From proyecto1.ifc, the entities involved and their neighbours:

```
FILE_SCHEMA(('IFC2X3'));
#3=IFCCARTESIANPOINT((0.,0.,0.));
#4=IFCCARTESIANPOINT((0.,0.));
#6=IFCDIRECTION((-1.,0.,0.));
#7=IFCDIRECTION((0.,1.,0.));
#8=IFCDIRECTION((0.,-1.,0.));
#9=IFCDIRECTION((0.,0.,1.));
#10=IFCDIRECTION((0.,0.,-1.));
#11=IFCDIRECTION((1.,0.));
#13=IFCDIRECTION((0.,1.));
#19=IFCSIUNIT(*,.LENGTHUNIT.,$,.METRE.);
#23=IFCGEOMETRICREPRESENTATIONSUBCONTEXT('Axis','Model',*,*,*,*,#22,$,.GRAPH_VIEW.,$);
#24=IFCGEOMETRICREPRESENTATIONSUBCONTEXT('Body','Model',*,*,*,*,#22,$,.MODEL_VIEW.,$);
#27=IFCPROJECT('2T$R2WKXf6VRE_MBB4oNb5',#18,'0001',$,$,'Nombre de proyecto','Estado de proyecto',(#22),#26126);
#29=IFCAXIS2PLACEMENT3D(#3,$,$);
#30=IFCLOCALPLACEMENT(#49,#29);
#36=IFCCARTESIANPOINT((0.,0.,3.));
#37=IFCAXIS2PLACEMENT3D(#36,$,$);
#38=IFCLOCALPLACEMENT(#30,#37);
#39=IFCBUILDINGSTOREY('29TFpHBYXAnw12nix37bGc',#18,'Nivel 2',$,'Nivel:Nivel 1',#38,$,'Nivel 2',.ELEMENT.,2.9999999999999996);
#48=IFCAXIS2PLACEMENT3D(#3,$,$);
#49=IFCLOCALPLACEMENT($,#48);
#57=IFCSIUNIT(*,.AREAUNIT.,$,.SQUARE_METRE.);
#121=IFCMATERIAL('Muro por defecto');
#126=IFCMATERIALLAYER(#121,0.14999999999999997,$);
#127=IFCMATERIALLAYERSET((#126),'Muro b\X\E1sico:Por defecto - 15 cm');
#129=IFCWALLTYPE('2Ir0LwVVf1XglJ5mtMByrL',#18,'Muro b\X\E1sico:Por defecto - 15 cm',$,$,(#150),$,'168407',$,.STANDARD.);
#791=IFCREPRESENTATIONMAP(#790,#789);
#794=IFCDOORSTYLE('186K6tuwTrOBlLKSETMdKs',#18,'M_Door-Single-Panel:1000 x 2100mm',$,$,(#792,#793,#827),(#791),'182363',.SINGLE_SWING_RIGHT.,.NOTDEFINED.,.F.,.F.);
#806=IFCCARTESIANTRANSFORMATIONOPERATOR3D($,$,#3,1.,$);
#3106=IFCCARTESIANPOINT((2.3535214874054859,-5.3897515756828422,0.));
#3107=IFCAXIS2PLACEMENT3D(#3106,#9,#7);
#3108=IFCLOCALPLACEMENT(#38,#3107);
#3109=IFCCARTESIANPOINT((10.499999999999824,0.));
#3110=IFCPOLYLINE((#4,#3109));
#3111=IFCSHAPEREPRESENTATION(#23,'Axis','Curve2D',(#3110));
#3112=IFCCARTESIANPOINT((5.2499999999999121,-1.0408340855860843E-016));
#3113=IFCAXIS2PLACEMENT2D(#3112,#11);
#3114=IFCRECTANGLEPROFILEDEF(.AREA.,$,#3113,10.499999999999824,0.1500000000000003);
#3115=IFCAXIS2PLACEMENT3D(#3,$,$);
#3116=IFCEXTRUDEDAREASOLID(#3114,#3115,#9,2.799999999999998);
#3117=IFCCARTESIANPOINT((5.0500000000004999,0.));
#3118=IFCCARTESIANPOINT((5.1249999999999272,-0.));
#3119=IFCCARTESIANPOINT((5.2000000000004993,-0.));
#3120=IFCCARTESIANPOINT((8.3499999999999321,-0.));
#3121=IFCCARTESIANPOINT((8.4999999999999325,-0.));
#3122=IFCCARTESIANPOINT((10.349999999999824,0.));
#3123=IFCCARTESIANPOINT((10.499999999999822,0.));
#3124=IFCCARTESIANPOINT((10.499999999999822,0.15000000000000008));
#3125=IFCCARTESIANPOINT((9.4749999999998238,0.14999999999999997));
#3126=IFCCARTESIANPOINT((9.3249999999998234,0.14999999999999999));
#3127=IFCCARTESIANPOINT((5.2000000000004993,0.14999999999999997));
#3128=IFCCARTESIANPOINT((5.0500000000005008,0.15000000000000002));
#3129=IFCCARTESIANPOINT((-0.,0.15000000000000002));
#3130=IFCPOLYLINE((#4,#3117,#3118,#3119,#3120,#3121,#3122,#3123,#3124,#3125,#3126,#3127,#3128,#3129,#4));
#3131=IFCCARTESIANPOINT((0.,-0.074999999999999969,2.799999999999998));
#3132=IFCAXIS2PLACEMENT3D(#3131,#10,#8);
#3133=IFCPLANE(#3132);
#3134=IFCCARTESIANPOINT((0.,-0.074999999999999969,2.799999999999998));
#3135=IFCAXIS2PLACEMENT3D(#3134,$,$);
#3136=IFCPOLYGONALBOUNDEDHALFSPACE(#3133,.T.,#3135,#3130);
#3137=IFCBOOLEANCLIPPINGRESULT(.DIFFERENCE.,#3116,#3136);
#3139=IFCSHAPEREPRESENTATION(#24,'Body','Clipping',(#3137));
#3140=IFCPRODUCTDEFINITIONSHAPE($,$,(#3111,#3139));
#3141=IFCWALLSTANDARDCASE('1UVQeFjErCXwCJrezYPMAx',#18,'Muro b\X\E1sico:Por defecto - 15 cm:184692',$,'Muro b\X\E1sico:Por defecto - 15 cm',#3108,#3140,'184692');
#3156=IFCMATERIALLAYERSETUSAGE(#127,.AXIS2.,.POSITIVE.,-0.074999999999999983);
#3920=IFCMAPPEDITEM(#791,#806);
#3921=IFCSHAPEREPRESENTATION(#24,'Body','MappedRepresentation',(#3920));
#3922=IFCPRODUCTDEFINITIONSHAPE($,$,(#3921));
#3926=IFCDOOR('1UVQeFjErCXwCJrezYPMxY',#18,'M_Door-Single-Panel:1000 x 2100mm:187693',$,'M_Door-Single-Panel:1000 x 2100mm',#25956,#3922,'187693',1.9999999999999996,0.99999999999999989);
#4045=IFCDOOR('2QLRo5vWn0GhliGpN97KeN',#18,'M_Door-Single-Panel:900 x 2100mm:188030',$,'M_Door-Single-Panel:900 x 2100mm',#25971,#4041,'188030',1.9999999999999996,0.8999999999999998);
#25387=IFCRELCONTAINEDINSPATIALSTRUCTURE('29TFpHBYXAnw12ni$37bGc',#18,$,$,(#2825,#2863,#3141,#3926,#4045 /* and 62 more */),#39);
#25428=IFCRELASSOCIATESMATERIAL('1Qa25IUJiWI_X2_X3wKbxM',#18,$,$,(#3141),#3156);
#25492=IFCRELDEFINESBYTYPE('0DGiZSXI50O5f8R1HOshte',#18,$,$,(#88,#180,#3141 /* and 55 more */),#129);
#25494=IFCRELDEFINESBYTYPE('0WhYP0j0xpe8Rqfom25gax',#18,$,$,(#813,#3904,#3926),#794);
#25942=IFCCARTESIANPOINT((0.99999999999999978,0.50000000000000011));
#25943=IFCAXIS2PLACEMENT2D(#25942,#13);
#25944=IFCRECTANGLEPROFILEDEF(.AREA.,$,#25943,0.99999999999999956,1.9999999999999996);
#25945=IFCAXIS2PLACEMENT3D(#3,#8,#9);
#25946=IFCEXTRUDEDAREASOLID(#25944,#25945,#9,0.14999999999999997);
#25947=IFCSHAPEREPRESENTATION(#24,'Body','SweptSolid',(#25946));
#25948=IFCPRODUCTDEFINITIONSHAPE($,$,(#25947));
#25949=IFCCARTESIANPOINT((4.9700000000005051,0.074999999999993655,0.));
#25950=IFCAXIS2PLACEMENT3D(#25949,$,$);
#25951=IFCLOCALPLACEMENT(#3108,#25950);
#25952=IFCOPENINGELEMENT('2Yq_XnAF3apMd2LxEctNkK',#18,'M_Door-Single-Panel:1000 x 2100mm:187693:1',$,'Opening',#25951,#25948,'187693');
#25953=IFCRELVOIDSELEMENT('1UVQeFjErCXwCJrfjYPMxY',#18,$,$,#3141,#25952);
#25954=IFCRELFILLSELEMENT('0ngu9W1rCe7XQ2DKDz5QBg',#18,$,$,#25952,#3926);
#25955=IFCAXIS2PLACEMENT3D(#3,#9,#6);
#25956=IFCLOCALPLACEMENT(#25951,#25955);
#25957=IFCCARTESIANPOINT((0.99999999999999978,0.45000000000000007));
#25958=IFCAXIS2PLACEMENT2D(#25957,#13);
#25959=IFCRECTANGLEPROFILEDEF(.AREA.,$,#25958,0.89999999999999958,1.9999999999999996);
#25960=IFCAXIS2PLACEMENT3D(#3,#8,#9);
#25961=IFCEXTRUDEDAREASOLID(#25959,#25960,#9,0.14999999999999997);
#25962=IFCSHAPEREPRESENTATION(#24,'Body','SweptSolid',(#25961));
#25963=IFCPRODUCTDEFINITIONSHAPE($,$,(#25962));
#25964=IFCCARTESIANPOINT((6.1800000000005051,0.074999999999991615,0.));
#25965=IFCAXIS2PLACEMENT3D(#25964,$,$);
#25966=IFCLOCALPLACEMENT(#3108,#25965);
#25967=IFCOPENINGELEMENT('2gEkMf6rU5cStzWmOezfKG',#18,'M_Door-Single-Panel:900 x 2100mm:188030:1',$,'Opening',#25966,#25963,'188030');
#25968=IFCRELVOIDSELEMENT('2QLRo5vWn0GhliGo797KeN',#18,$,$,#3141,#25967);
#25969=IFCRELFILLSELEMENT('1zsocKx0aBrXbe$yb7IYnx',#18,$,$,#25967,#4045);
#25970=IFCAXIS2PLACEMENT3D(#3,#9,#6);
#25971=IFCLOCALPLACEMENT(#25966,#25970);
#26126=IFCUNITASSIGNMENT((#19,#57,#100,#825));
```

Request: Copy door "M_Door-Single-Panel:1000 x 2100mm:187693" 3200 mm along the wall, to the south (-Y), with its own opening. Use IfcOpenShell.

```python
import ifcopenshell
import ifcopenshell.api.feature
import ifcopenshell.api.geometry
import ifcopenshell.api.root
import ifcopenshell.geom
import ifcopenshell.util.element
import ifcopenshell.util.placement
import ifcopenshell.util.shape
import ifcopenshell.util.unit

model = ifcopenshell.open("proyecto1.ifc")
unit_scale = ifcopenshell.util.unit.calculate_unit_scale(model)
settings = ifcopenshell.geom.settings()


def volume(element):
    """Net volume in cubic metres, openings subtracted."""
    shape = ifcopenshell.geom.create_shape(settings, element)
    return ifcopenshell.util.shape.get_volume(shape.geometry)


def reuse_history(source, copy):
    """copy_class also copies each property set's owner history, people and application; keep the originals."""
    for rel in copy.IsDefinedBy:
        if rel.is_a("IfcRelDefinesByProperties") and (history := rel.RelatingPropertyDefinition.OwnerHistory):
            rel.RelatingPropertyDefinition.OwnerHistory = source.OwnerHistory
            ifcopenshell.util.element.remove_deep2(model, history)


door = model.by_id(3926)
opening = door.FillsVoids[0].RelatingOpeningElement
wall = opening.VoidsElements[0].RelatingBuildingElement
before = volume(wall)
shift = ifcopenshell.util.placement.get_local_placement(wall.ObjectPlacement)[:3, 0] * -3.2 / unit_scale

# copy_class copies the void relationship, type, container and properties, but no geometry.
new_opening = ifcopenshell.api.root.copy_class(model, product=opening)
new_opening.Representation = ifcopenshell.util.element.copy_deep(
    model, opening.Representation, exclude=["IfcGeometricRepresentationContext", "IfcRepresentationMap"]
)
new_opening.Name = "M_Door-Single-Panel:1000 x 2100mm"
new_opening.Tag = None
new_door = ifcopenshell.api.root.copy_class(model, product=door)
new_door.Representation = ifcopenshell.util.element.copy_deep(
    model, door.Representation, exclude=["IfcGeometricRepresentationContext", "IfcRepresentationMap"]
)
new_door.Name = "M_Door-Single-Panel:1000 x 2100mm"
new_door.Tag = None
reuse_history(door, new_door)
fills = ifcopenshell.api.feature.add_filling(model, opening=new_opening, element=new_door)
fills.OwnerHistory = new_door.OwnerHistory  # required in IFC2X3

for old, new in ((opening, new_opening), (door, new_door)):
    matrix = ifcopenshell.util.placement.get_local_placement(old.ObjectPlacement)
    matrix[:3, 3] += shift
    ifcopenshell.api.geometry.edit_object_placement(model, product=new, matrix=matrix, is_si=False)

after = volume(wall)

print(f"wall volume {before:.3f} -> {after:.3f} m3")

model.write("proyecto1_rev.ifc")
```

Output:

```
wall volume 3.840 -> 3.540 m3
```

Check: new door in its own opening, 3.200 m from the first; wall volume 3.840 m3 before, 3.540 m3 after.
